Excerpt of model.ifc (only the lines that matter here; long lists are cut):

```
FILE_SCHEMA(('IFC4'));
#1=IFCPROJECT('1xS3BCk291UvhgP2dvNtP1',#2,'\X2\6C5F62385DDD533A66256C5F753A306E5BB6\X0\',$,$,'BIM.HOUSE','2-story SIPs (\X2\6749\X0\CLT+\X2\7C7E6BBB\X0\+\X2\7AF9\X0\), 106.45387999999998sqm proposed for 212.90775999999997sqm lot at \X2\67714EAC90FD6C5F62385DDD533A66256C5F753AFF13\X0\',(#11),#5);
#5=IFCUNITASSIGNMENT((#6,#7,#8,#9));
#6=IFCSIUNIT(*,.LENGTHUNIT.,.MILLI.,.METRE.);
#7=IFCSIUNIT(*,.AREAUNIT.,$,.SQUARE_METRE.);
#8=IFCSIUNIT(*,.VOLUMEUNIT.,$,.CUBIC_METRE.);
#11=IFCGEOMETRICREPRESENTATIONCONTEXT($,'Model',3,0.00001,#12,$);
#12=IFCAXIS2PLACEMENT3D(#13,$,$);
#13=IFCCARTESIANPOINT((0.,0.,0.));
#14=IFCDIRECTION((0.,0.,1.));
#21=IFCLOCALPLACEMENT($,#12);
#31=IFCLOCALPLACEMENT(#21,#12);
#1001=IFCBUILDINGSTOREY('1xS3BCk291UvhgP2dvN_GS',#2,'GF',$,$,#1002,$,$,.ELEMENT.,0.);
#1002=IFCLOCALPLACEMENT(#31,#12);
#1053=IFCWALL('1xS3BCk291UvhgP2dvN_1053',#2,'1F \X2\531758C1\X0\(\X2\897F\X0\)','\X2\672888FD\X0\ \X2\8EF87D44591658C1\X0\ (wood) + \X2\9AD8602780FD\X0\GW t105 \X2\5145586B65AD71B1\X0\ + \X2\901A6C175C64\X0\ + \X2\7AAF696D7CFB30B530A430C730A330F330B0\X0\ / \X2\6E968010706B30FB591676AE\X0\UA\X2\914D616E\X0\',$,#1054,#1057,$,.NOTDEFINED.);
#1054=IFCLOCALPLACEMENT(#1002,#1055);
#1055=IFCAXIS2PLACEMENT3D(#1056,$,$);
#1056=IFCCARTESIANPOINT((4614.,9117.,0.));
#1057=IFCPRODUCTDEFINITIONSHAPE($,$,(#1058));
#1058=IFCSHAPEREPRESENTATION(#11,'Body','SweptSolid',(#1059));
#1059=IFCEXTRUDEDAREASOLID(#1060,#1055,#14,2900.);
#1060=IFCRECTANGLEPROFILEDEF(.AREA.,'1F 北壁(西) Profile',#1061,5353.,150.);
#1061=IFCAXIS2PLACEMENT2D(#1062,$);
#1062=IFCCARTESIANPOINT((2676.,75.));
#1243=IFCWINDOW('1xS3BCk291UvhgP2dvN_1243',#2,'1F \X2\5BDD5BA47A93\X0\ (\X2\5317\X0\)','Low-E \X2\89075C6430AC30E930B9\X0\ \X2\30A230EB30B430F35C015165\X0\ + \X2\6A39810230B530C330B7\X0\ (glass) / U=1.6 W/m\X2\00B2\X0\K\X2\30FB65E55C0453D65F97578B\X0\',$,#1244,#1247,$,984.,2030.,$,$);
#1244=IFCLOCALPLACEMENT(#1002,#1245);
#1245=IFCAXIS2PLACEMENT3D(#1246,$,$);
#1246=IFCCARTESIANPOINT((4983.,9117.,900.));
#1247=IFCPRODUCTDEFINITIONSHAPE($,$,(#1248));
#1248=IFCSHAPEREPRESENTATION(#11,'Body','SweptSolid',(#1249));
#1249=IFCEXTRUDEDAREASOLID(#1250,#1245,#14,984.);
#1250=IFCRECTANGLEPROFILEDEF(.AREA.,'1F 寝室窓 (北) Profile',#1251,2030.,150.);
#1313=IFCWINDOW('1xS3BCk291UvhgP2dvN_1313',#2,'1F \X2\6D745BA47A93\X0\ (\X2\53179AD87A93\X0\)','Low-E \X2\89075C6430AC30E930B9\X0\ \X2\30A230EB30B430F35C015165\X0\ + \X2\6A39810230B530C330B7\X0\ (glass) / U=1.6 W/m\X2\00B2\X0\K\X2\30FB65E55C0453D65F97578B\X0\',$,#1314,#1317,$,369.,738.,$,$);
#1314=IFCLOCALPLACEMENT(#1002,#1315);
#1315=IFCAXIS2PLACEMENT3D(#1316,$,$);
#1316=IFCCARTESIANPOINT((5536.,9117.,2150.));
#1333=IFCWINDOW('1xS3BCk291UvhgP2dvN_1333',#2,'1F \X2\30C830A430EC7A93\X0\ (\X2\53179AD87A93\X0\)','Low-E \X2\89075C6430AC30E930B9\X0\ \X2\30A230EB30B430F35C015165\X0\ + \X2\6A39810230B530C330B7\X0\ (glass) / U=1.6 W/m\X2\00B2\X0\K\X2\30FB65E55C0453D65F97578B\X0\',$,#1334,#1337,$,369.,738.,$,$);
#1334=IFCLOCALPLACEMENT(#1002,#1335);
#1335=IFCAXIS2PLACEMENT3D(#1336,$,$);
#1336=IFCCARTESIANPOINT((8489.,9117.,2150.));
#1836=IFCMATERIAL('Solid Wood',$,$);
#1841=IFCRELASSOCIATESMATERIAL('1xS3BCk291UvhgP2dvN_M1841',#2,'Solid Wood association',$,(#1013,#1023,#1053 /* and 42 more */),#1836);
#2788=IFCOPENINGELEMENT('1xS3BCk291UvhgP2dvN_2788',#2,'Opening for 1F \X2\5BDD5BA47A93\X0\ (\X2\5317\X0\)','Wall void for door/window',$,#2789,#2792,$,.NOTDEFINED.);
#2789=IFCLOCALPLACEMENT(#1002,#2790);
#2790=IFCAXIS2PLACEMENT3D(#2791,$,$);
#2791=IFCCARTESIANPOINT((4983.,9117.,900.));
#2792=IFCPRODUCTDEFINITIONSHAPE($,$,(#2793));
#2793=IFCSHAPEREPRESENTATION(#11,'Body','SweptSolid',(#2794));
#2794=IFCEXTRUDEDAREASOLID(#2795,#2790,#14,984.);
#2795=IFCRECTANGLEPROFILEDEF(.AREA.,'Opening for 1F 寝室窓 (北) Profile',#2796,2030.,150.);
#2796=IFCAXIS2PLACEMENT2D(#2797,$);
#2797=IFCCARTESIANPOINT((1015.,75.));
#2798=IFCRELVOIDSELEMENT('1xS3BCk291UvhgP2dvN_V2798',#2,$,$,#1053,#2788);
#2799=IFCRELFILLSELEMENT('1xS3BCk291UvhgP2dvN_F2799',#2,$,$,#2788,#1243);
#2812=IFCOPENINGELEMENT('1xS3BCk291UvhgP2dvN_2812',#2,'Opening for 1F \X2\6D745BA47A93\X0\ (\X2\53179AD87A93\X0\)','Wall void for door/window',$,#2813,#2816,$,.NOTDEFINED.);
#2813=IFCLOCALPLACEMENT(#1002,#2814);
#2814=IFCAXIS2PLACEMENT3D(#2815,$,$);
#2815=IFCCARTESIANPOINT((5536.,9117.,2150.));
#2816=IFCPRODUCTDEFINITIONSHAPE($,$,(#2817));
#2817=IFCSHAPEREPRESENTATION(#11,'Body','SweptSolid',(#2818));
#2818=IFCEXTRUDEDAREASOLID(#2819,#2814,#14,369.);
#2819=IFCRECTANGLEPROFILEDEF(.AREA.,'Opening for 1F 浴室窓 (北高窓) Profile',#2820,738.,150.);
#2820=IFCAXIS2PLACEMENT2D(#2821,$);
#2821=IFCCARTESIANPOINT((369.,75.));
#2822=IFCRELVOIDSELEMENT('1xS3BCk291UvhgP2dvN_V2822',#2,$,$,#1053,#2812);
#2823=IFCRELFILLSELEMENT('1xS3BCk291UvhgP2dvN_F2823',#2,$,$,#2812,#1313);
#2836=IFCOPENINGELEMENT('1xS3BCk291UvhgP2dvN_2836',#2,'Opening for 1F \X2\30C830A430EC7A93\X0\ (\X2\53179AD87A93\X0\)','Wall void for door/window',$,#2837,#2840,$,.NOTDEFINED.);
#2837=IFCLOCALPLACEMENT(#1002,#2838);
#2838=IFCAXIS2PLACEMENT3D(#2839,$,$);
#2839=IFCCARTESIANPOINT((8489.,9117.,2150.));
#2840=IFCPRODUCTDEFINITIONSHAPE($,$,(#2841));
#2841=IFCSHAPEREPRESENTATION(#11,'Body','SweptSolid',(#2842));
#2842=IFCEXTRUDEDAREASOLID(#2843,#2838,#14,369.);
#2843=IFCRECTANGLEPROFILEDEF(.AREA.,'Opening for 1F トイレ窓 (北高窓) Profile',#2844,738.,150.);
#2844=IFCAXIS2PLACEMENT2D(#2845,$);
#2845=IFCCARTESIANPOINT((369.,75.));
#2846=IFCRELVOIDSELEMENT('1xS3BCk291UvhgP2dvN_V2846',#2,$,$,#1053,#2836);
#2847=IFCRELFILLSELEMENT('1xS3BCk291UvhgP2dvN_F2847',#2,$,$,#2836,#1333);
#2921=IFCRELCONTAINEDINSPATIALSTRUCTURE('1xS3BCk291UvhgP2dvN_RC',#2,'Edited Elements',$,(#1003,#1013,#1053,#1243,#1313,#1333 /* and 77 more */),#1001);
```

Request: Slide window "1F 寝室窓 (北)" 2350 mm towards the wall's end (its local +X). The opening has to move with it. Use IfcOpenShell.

```python
import ifcopenshell
import ifcopenshell.api.geometry
import ifcopenshell.util.placement
import ifcopenshell.util.unit

model = ifcopenshell.open("model.ifc")
unit_scale = ifcopenshell.util.unit.calculate_unit_scale(model)

window = model.by_guid("1xS3BCk291UvhgP2dvN_1243")
opening = window.FillsVoids[0].RelatingOpeningElement
wall = opening.VoidsElements[0].RelatingBuildingElement

wall_matrix = ifcopenshell.util.placement.get_local_placement(wall.ObjectPlacement)
shift = wall_matrix[:3, 0] * 2.35 / unit_scale
before = ifcopenshell.util.placement.get_local_placement(window.ObjectPlacement)[:3, 3].copy()

# The window is not placed relative to its opening, so move both.
for product in (opening, window):
    matrix = ifcopenshell.util.placement.get_local_placement(product.ObjectPlacement)
    matrix[:3, 3] += shift
    ifcopenshell.api.geometry.edit_object_placement(model, product=product, matrix=matrix, is_si=False)

after = ifcopenshell.util.placement.get_local_placement(window.ObjectPlacement)[:3, 3]
print("window moved by", (after - before).round(3) + 0.0)

model.write("model-out.ifc")
```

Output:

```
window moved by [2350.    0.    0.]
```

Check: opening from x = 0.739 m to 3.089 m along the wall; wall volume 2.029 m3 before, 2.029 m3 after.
